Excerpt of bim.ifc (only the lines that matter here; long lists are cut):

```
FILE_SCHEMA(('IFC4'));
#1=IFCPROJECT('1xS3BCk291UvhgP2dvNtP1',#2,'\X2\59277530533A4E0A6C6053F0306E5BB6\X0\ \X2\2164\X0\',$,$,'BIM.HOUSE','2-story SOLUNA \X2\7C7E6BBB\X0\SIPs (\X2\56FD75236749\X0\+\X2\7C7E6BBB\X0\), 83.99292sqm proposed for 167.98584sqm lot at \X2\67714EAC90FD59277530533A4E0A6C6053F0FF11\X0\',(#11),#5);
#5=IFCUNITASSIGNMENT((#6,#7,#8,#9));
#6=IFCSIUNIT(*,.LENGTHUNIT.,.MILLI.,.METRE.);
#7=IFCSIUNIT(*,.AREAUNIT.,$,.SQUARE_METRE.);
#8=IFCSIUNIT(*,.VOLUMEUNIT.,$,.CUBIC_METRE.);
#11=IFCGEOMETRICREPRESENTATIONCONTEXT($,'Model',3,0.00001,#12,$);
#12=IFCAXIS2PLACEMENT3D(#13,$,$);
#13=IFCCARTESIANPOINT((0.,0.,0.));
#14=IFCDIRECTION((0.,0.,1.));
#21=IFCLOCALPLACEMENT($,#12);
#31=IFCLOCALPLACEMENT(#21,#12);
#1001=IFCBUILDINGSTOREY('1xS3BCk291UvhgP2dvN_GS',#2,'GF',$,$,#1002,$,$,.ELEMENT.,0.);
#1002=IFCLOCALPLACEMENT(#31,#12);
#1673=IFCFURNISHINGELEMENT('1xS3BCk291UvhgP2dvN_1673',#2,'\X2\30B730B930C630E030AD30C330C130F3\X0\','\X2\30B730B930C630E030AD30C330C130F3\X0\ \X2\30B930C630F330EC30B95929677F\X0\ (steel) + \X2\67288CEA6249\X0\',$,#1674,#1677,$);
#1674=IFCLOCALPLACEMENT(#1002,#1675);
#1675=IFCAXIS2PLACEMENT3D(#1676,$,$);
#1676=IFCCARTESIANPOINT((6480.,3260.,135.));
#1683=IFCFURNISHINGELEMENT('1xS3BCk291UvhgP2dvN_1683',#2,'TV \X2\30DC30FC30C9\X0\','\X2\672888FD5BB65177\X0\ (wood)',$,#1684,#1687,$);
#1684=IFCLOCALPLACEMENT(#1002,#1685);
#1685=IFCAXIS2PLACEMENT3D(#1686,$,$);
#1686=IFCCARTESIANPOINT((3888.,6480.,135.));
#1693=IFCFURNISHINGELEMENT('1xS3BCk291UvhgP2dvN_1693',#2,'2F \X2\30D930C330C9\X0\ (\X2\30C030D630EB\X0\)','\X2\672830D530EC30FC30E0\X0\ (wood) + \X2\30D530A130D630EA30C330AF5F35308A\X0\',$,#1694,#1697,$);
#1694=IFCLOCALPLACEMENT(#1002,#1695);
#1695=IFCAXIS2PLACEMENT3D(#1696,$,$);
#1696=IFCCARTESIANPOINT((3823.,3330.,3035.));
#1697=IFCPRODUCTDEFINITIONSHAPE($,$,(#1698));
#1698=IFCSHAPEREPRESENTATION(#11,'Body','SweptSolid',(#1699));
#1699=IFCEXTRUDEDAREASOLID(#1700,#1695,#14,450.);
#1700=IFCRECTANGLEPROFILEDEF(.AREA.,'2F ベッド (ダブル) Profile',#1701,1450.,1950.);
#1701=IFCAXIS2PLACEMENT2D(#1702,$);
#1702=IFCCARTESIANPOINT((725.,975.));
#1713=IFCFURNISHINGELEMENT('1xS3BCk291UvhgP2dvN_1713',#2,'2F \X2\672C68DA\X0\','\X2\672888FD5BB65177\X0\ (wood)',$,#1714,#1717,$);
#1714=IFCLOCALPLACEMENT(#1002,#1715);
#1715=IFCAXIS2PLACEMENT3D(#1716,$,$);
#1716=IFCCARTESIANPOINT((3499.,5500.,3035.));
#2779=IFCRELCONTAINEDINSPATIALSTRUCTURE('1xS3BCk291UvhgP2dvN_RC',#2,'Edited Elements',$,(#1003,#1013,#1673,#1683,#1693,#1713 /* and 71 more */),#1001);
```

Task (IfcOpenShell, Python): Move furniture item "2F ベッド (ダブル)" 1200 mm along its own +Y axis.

```python
import ifcopenshell
import ifcopenshell.api.geometry
import ifcopenshell.util.placement
import ifcopenshell.util.unit

model = ifcopenshell.open("bim.ifc")
unit_scale = ifcopenshell.util.unit.calculate_unit_scale(model)

item = model.by_guid("1xS3BCk291UvhgP2dvN_1693")
matrix = ifcopenshell.util.placement.get_local_placement(item.ObjectPlacement)
matrix[:3, 3] += matrix[:3, 1] * 1.2 / unit_scale
ifcopenshell.api.geometry.edit_object_placement(model, product=item, matrix=matrix, is_si=False)

print(ifcopenshell.util.placement.get_local_placement(item.ObjectPlacement).round(3) + 0.0)

model.write("bim_v2.ifc")
```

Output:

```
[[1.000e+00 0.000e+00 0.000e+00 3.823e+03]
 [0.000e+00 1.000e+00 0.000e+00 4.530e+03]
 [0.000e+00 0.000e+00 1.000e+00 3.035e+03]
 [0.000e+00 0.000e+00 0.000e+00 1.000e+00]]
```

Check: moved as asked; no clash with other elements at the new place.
